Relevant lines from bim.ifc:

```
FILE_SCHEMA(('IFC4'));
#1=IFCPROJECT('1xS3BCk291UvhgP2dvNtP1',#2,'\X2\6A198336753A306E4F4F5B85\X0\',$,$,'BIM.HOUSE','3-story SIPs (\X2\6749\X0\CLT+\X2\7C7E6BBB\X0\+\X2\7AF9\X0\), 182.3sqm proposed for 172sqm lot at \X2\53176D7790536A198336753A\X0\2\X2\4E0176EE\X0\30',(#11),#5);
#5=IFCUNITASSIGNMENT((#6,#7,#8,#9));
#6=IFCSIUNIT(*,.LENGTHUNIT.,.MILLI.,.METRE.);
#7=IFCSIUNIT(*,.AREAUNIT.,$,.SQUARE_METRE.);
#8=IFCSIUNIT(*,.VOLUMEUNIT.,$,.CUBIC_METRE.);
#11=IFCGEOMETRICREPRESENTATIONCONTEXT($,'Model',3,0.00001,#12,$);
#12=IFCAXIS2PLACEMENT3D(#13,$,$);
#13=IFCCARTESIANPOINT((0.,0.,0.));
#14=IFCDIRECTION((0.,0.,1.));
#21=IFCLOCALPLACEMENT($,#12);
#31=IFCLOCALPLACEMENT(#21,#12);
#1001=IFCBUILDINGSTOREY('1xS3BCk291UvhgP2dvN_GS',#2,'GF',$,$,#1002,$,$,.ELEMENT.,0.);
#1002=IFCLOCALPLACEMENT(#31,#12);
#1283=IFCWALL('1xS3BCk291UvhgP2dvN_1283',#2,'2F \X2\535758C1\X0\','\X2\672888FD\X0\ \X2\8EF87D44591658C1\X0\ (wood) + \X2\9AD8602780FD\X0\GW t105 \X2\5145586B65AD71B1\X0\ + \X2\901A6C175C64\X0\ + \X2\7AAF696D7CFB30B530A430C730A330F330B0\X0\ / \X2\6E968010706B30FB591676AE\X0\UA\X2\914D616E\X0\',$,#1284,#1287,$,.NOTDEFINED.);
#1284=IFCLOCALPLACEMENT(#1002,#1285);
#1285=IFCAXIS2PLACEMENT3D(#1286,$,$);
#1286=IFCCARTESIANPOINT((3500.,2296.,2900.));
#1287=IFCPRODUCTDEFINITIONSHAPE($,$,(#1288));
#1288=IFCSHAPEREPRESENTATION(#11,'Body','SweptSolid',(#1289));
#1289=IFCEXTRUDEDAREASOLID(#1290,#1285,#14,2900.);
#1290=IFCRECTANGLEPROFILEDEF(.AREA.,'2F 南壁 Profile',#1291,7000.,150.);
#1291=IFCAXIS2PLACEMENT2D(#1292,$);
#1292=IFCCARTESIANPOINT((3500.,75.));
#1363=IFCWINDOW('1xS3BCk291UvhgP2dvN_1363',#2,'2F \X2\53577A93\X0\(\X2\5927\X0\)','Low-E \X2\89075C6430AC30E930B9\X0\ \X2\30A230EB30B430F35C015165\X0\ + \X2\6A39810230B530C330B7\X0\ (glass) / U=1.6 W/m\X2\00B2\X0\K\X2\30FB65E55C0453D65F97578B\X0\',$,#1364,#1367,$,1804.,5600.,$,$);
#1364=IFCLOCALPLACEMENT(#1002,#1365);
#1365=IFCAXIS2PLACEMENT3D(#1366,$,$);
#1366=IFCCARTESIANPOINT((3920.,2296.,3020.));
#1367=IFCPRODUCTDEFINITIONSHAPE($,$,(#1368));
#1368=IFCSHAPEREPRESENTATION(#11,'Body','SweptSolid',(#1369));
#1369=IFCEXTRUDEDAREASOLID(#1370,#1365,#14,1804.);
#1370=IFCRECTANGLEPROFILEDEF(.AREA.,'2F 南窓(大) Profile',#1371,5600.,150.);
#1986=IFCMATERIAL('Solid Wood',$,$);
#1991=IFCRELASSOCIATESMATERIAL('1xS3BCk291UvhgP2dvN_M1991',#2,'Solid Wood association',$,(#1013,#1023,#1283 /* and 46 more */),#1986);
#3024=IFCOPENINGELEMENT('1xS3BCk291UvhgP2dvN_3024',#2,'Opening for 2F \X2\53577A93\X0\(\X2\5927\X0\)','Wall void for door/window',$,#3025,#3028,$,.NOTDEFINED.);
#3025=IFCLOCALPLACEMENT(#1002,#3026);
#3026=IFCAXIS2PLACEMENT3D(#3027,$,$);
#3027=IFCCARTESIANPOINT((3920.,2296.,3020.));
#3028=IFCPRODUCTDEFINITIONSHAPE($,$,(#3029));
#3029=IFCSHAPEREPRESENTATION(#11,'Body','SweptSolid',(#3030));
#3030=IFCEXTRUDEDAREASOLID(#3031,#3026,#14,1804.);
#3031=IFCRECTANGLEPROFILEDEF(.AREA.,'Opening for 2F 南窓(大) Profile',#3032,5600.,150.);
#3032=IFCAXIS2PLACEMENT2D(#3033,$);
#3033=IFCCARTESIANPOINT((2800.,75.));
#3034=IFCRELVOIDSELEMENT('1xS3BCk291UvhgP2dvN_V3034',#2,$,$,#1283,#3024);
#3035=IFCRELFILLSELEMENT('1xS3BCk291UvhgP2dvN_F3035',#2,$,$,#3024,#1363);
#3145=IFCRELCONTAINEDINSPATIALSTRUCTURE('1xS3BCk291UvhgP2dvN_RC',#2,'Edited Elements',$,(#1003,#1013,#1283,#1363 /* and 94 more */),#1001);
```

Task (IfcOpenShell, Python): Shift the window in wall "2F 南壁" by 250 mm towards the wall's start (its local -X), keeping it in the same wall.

```python
import ifcopenshell
import ifcopenshell.api.geometry
import ifcopenshell.util.placement

model = ifcopenshell.open("bim.ifc")

window = model.by_guid("1xS3BCk291UvhgP2dvN_1363")
opening = window.FillsVoids[0].RelatingOpeningElement
wall = opening.VoidsElements[0].RelatingBuildingElement

wall_matrix = ifcopenshell.util.placement.get_local_placement(wall.ObjectPlacement)
shift = wall_matrix[:3, 0] * -250.0
before = ifcopenshell.util.placement.get_local_placement(window.ObjectPlacement)[:3, 3].copy()

# The window is not placed relative to its opening, so move both.
for product in (opening, window):
    matrix = ifcopenshell.util.placement.get_local_placement(product.ObjectPlacement)
    matrix[:3, 3] += shift
    ifcopenshell.api.geometry.edit_object_placement(model, product=product, matrix=matrix, is_si=False)

after = ifcopenshell.util.placement.get_local_placement(window.ObjectPlacement)[:3, 3]
print("window moved by", (after - before).round(3) + 0.0)

model.write("bim_edited.ifc")
```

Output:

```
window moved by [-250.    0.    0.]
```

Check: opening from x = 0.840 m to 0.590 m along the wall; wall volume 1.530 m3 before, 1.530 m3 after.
